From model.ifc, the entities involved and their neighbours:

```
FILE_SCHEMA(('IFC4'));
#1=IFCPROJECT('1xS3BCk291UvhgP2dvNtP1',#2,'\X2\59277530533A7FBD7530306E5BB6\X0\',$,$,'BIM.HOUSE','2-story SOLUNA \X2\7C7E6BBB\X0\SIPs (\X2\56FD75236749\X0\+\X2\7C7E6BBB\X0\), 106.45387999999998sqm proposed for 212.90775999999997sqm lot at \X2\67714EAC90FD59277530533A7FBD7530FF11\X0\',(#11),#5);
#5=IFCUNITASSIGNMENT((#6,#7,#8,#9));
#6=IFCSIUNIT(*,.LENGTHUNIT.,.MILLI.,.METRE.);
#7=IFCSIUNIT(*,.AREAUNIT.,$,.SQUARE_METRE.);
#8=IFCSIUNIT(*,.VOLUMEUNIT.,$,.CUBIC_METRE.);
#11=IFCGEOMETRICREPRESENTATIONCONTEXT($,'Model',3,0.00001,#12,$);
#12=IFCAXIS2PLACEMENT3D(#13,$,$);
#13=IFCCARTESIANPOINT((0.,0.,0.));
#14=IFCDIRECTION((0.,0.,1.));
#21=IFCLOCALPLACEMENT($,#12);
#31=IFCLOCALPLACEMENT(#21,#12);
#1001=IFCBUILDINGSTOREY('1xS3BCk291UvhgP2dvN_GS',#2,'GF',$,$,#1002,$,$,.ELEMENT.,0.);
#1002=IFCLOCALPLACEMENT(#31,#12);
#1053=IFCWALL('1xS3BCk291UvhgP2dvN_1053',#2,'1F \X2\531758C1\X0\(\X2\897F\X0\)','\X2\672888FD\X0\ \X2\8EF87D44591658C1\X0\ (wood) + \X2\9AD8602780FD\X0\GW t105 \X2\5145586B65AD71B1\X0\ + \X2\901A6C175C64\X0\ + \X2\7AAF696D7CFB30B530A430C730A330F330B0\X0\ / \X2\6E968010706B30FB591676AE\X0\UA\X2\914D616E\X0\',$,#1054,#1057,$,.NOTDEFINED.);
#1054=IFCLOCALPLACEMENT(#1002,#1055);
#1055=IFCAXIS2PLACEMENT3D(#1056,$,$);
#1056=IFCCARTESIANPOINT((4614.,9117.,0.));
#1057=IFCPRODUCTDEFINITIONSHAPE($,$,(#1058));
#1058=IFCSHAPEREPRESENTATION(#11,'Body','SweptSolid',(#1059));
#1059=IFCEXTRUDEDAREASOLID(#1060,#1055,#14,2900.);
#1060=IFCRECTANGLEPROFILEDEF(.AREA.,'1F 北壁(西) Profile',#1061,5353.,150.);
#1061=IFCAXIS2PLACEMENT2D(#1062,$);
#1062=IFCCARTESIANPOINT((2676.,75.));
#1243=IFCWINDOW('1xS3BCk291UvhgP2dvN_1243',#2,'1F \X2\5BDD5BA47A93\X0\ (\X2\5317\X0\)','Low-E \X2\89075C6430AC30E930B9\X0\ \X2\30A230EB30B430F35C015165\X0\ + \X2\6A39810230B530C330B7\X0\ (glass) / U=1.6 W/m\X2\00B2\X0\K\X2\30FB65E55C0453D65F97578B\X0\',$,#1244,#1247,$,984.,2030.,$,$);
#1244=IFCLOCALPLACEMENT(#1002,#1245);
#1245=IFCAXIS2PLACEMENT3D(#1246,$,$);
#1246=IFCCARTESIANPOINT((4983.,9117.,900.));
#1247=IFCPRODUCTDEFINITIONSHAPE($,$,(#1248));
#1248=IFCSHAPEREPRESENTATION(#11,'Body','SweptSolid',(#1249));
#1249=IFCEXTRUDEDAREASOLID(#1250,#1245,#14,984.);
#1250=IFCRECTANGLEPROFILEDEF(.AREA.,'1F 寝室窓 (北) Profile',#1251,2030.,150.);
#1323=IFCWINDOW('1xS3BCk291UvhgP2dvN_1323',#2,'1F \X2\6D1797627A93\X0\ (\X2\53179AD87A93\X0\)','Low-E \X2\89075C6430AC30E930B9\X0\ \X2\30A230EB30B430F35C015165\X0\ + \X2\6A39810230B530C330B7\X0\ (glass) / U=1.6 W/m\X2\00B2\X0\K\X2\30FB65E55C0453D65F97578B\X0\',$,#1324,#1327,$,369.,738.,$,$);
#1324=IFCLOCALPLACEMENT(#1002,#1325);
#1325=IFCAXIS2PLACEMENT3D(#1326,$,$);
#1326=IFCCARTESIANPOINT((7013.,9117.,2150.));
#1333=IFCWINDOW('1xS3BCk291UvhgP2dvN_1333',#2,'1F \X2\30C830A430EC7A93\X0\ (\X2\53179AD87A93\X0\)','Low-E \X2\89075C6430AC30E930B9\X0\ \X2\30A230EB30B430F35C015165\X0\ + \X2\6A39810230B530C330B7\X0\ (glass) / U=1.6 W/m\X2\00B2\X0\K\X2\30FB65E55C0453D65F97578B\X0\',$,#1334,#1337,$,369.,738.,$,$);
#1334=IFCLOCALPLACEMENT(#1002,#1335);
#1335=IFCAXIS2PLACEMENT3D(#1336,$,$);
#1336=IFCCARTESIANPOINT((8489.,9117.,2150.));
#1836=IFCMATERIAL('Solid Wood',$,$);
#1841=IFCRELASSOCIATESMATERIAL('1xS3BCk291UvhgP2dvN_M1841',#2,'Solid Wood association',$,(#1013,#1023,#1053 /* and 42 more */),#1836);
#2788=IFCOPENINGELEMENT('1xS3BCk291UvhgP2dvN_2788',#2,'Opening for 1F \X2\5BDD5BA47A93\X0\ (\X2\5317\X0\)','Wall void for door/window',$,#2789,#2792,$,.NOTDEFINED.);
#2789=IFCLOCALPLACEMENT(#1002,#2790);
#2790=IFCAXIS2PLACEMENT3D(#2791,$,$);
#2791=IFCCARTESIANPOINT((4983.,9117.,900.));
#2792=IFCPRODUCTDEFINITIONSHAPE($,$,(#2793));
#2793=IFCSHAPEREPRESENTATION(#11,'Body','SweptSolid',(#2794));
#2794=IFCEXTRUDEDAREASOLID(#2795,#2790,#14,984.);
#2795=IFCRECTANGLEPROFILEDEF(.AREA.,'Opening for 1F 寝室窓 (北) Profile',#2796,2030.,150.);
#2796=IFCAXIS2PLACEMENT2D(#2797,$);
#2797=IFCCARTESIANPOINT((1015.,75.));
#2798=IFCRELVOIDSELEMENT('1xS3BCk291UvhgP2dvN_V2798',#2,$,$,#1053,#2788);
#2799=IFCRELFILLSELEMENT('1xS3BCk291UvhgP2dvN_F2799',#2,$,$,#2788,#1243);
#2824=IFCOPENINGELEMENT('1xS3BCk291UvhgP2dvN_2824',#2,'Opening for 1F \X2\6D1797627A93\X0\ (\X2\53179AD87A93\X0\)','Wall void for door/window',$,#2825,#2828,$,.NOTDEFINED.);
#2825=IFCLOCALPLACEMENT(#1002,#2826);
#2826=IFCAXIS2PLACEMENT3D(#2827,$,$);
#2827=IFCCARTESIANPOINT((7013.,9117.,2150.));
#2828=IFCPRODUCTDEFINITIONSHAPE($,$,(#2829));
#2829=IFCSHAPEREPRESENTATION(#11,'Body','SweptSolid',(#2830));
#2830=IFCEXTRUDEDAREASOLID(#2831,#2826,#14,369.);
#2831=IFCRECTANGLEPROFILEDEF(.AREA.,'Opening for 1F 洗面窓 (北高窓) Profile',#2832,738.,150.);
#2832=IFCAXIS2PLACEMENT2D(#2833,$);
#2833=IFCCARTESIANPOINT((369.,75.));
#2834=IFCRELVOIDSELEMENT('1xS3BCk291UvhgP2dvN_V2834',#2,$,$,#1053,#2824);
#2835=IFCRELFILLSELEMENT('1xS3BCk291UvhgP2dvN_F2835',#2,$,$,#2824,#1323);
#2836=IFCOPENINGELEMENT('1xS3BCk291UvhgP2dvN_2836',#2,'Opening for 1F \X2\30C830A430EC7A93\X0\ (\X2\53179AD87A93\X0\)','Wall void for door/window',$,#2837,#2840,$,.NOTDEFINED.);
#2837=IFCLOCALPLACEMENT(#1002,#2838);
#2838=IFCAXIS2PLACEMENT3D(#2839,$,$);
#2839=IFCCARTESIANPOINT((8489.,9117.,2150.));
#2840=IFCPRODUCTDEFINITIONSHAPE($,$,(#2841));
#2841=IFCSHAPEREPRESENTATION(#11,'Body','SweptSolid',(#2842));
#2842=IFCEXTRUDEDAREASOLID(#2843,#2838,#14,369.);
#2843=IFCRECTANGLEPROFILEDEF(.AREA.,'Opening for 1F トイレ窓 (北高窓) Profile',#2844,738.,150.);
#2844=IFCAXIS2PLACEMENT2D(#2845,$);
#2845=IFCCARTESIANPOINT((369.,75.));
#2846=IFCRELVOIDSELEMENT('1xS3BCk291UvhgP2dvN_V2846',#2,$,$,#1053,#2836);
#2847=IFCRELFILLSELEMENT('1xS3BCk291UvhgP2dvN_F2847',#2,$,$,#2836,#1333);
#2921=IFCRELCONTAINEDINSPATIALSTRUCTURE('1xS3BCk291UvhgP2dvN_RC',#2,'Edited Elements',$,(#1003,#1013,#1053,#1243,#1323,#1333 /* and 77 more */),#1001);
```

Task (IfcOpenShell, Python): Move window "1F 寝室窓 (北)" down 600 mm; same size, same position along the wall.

```python
import numpy as np
import ifcopenshell
import ifcopenshell.api.geometry
import ifcopenshell.util.placement
import ifcopenshell.util.unit

model = ifcopenshell.open("model.ifc")
unit_scale = ifcopenshell.util.unit.calculate_unit_scale(model)

window = model.by_guid("1xS3BCk291UvhgP2dvN_1243")
opening = window.FillsVoids[0].RelatingOpeningElement
dz = -0.6 / unit_scale

shift = np.array([0.0, 0.0, dz])
# The window is not placed relative to its opening, so move both.
for product in (opening, window):
    matrix = ifcopenshell.util.placement.get_local_placement(product.ObjectPlacement)
    matrix[:3, 3] += shift
    ifcopenshell.api.geometry.edit_object_placement(model, product=product, matrix=matrix, is_si=False)

print(f"moved by {dz * unit_scale:+.3f} m")

model.write("model_rev.ifc")
```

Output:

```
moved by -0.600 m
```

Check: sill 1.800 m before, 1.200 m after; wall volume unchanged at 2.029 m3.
